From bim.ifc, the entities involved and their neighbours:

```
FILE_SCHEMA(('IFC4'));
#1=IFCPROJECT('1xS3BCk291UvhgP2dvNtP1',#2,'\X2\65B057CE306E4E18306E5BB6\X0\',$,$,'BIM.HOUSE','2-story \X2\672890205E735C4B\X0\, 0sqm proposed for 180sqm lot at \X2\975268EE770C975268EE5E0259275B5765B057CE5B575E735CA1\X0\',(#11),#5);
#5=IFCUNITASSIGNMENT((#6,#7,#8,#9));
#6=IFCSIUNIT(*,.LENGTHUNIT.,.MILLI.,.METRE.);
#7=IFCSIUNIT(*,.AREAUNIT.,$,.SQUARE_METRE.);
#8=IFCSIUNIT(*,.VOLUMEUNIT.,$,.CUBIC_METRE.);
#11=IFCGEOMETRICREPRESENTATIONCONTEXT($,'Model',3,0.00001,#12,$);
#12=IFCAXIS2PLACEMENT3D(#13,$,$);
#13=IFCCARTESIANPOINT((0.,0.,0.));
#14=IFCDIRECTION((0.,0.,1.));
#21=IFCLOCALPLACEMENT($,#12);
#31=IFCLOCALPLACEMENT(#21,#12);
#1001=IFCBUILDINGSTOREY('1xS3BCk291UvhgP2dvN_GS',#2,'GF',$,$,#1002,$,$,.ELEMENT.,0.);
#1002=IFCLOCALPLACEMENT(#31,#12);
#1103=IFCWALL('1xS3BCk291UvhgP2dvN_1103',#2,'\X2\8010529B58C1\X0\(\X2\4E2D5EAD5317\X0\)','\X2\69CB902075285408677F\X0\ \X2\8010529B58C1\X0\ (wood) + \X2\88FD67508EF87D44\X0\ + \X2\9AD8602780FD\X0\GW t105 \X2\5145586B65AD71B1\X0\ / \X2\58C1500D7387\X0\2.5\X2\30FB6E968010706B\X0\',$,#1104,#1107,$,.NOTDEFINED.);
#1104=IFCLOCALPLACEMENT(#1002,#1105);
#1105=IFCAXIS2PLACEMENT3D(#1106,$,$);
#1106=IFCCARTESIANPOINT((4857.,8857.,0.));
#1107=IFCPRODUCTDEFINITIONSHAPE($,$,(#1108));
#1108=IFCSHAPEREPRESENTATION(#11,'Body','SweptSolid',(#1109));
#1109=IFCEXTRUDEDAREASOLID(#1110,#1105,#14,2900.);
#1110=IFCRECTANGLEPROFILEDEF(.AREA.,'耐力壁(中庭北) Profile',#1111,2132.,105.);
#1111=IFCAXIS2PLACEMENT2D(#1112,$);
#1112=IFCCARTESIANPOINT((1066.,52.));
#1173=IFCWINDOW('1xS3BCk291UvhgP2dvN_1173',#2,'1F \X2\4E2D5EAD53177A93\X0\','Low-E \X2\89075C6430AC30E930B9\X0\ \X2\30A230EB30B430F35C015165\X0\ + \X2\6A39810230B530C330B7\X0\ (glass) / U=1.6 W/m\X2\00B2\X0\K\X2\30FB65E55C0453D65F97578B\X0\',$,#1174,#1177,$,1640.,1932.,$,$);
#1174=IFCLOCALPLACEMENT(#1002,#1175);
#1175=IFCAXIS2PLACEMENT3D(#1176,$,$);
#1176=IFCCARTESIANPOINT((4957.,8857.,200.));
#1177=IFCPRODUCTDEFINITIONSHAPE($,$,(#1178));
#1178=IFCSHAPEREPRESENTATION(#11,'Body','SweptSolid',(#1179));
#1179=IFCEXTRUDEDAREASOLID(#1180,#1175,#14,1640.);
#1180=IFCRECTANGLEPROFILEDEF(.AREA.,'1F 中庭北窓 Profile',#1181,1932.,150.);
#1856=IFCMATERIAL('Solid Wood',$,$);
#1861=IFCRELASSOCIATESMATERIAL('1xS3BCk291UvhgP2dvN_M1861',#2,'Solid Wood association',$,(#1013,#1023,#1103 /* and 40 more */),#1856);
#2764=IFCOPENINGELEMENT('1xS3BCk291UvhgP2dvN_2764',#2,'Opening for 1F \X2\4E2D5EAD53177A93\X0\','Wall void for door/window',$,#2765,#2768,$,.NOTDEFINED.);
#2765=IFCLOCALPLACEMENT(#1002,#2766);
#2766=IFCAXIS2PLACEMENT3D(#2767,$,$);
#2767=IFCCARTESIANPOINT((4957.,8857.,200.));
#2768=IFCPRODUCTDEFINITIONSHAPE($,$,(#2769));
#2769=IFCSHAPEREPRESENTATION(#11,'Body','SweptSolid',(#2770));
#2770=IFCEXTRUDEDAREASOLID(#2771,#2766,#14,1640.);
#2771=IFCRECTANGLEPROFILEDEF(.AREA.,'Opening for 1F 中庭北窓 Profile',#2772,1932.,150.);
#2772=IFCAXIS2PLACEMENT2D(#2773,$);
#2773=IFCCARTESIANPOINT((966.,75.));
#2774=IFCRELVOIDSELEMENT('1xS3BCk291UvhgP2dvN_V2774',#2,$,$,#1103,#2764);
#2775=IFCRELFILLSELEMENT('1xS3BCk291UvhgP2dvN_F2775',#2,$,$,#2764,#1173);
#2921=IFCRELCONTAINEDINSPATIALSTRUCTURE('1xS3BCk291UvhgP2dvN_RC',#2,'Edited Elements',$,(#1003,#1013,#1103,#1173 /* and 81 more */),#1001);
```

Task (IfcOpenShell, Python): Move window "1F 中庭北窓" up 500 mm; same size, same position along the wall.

```python
import numpy as np
import ifcopenshell
import ifcopenshell.api.geometry
import ifcopenshell.util.placement
import ifcopenshell.util.unit

model = ifcopenshell.open("bim.ifc")
unit_scale = ifcopenshell.util.unit.calculate_unit_scale(model)

window = model.by_guid("1xS3BCk291UvhgP2dvN_1173")
opening = window.FillsVoids[0].RelatingOpeningElement
dz = 500.0

shift = np.array([0.0, 0.0, dz])
# The window is not placed relative to its opening, so move both.
for product in (opening, window):
    matrix = ifcopenshell.util.placement.get_local_placement(product.ObjectPlacement)
    matrix[:3, 3] += shift
    ifcopenshell.api.geometry.edit_object_placement(model, product=product, matrix=matrix, is_si=False)

print(f"moved by {dz * unit_scale:+.3f} m")

model.write("bim_updated.ifc")
```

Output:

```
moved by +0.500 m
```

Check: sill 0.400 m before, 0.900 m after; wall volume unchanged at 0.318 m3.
